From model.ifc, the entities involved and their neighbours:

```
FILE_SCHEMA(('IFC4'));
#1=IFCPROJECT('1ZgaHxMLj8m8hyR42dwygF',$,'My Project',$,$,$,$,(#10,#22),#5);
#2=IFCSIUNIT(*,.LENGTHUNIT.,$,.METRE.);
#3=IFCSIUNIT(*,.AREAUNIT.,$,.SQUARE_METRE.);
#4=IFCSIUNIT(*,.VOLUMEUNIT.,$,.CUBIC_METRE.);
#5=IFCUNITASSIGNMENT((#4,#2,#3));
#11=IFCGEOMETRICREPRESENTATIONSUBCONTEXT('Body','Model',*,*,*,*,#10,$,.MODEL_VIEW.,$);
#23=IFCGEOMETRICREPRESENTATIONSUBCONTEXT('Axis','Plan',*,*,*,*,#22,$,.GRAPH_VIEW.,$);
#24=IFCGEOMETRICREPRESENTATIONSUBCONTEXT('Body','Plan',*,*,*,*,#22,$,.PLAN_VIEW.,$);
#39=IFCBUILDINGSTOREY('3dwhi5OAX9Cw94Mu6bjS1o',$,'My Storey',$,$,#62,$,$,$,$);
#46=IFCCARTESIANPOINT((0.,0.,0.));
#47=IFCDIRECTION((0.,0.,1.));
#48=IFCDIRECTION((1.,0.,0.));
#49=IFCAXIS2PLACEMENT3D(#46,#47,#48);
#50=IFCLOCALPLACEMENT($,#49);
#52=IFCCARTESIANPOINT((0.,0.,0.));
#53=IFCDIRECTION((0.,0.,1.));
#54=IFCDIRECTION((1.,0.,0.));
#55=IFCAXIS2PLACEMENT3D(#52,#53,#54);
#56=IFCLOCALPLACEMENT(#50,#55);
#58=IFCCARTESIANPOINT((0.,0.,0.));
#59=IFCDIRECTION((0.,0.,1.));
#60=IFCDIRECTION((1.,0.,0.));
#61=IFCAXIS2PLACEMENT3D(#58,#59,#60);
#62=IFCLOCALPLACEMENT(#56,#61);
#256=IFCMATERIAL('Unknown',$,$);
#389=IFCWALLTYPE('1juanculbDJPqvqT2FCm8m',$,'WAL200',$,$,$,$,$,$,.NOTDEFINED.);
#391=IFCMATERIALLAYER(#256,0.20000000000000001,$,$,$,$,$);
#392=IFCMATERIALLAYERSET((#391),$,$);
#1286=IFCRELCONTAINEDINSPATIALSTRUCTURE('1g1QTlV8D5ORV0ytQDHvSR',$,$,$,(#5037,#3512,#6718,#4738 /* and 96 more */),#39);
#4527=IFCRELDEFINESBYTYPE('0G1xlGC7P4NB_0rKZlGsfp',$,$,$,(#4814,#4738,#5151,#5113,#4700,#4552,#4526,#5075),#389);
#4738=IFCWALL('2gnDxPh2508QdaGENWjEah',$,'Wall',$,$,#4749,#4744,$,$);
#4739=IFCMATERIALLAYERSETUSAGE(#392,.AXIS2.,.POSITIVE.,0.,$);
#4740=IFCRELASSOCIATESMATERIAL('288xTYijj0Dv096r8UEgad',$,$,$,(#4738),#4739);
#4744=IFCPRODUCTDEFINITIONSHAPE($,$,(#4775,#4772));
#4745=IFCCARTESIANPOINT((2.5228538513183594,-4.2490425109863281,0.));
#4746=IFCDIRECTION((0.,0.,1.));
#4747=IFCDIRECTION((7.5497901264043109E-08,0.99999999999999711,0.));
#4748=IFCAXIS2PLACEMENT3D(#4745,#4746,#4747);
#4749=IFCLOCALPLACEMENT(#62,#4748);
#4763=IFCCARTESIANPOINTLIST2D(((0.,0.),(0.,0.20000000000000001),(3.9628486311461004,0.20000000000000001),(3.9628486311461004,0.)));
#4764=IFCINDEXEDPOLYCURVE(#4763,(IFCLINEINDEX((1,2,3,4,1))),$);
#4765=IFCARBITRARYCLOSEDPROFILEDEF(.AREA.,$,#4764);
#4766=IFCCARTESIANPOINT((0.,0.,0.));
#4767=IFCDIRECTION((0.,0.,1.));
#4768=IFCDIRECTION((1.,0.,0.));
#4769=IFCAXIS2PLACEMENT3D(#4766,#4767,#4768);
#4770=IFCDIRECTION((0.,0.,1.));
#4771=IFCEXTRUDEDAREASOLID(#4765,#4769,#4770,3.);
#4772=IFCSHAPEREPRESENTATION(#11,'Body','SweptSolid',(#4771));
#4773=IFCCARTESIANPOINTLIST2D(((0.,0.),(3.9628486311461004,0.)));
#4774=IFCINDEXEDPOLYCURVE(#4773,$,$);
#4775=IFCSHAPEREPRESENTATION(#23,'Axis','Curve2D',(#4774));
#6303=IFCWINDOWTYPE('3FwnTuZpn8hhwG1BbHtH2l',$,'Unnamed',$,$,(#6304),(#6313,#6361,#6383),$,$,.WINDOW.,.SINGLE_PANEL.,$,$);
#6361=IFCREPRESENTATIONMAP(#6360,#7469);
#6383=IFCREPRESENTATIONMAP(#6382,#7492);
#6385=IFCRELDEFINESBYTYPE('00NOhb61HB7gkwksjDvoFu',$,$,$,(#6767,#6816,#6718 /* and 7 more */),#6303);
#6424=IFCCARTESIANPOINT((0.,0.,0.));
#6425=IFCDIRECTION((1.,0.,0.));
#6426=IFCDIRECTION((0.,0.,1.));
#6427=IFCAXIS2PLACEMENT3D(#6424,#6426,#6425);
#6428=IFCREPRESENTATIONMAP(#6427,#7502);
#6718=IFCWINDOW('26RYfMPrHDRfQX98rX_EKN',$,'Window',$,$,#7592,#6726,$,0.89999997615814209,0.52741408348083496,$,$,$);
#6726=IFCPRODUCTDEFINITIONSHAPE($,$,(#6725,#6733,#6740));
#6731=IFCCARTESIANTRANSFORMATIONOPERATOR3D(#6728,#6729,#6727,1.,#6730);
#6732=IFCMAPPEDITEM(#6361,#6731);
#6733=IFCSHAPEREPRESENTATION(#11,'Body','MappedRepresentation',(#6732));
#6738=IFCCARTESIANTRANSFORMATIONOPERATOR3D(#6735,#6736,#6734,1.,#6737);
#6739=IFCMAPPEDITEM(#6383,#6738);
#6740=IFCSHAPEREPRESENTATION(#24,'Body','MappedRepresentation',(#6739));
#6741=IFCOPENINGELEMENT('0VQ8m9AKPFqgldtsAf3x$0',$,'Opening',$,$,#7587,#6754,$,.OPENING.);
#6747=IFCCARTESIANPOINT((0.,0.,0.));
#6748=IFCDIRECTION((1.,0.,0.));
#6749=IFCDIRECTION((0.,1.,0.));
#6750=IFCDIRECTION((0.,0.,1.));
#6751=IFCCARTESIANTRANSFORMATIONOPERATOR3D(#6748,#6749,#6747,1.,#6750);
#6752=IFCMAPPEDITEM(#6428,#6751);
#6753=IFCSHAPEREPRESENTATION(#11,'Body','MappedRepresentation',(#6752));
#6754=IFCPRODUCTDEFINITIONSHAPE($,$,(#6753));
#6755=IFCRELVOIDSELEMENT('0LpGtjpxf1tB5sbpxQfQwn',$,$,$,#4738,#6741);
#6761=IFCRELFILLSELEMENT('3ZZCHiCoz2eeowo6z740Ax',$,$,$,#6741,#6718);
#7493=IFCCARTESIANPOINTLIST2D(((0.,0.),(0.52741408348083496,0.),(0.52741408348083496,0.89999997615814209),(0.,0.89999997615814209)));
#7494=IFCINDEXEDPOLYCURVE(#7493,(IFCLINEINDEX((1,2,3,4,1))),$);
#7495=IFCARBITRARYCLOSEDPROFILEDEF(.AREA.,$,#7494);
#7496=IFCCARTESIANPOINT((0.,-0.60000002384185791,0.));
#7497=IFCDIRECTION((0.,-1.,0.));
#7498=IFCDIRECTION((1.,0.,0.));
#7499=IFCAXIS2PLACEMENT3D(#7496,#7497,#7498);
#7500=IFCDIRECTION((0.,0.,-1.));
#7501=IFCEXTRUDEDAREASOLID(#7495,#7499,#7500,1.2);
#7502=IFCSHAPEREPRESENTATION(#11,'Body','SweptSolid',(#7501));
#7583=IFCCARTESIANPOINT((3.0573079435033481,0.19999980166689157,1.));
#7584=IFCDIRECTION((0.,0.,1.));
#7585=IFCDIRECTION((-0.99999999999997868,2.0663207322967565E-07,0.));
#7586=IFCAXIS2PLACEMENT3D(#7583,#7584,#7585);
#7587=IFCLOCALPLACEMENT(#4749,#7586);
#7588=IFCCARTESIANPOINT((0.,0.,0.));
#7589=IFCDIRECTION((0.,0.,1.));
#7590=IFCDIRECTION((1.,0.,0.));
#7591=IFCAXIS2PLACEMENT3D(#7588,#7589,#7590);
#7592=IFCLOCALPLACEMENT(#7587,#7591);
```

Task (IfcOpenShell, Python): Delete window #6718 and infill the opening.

```python
import ifcopenshell
import ifcopenshell.api.feature
import ifcopenshell.api.root
import ifcopenshell.geom
import ifcopenshell.util.shape

model = ifcopenshell.open("model.ifc")
settings = ifcopenshell.geom.settings()


def volume(element):
    """Net volume in cubic metres, openings subtracted."""
    shape = ifcopenshell.geom.create_shape(settings, element)
    return ifcopenshell.util.shape.get_volume(shape.geometry)


window = model.by_guid("26RYfMPrHDRfQX98rX_EKN")
opening = window.FillsVoids[0].RelatingOpeningElement
wall = opening.VoidsElements[0].RelatingBuildingElement
before = volume(wall)

ifcopenshell.api.root.remove_product(model, product=window)
ifcopenshell.api.feature.remove_feature(model, feature=opening)

after = volume(wall)

print(f"wall volume {before:.3f} -> {after:.3f} m3")

model.write("model-out.ifc")
```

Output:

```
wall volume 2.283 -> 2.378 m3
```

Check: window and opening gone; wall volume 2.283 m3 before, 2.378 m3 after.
